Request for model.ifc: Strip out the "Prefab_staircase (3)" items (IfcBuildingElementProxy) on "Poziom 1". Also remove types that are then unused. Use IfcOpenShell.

First a look at what the model holds.

```python
import ifcopenshell
import ifcopenshell.util.element

model = ifcopenshell.open("model.ifc")
print(model.schema)
storey = next(s for s in model.by_type("IfcBuildingStorey") if s.Name == "Poziom 1")
proxies = [e for e in ifcopenshell.util.element.get_decomposition(storey) if e.is_a("IfcBuildingElementProxy")]
seen = {}
for e in proxies:
    element_type = ifcopenshell.util.element.get_type(e)
    name = element_type.Name if element_type not in (None, e) else None
    seen[name] = seen.get(name, 0) + 1
for name, count in sorted(seen.items(), key=str):
    print(count, "x", name)
```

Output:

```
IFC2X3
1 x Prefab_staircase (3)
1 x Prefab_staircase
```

```python
import ifcopenshell
import ifcopenshell.api.root
import ifcopenshell.util.element

model = ifcopenshell.open("model.ifc")

storey = next(s for s in model.by_type("IfcBuildingStorey") if s.Name == "Poziom 1")
proxies = [e for e in ifcopenshell.util.element.get_decomposition(storey) if e.is_a("IfcBuildingElementProxy")]
targets = [e for e in proxies if (t := ifcopenshell.util.element.get_type(e)) not in (None, e) and t.Name == "Prefab_staircase (3)"]
types = {ifcopenshell.util.element.get_type(e) for e in targets} - {None, *targets}

for e in targets:
    ifcopenshell.api.root.remove_product(model, product=e)
print(len(targets), "removed")

unused = [t for t in types if not ifcopenshell.util.element.get_types(t)]
for t in unused:
    ifcopenshell.api.root.remove_product(model, product=t)
print(len(unused), "unused types removed")

model.write("model-out.ifc")
```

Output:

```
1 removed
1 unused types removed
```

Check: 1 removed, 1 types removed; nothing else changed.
